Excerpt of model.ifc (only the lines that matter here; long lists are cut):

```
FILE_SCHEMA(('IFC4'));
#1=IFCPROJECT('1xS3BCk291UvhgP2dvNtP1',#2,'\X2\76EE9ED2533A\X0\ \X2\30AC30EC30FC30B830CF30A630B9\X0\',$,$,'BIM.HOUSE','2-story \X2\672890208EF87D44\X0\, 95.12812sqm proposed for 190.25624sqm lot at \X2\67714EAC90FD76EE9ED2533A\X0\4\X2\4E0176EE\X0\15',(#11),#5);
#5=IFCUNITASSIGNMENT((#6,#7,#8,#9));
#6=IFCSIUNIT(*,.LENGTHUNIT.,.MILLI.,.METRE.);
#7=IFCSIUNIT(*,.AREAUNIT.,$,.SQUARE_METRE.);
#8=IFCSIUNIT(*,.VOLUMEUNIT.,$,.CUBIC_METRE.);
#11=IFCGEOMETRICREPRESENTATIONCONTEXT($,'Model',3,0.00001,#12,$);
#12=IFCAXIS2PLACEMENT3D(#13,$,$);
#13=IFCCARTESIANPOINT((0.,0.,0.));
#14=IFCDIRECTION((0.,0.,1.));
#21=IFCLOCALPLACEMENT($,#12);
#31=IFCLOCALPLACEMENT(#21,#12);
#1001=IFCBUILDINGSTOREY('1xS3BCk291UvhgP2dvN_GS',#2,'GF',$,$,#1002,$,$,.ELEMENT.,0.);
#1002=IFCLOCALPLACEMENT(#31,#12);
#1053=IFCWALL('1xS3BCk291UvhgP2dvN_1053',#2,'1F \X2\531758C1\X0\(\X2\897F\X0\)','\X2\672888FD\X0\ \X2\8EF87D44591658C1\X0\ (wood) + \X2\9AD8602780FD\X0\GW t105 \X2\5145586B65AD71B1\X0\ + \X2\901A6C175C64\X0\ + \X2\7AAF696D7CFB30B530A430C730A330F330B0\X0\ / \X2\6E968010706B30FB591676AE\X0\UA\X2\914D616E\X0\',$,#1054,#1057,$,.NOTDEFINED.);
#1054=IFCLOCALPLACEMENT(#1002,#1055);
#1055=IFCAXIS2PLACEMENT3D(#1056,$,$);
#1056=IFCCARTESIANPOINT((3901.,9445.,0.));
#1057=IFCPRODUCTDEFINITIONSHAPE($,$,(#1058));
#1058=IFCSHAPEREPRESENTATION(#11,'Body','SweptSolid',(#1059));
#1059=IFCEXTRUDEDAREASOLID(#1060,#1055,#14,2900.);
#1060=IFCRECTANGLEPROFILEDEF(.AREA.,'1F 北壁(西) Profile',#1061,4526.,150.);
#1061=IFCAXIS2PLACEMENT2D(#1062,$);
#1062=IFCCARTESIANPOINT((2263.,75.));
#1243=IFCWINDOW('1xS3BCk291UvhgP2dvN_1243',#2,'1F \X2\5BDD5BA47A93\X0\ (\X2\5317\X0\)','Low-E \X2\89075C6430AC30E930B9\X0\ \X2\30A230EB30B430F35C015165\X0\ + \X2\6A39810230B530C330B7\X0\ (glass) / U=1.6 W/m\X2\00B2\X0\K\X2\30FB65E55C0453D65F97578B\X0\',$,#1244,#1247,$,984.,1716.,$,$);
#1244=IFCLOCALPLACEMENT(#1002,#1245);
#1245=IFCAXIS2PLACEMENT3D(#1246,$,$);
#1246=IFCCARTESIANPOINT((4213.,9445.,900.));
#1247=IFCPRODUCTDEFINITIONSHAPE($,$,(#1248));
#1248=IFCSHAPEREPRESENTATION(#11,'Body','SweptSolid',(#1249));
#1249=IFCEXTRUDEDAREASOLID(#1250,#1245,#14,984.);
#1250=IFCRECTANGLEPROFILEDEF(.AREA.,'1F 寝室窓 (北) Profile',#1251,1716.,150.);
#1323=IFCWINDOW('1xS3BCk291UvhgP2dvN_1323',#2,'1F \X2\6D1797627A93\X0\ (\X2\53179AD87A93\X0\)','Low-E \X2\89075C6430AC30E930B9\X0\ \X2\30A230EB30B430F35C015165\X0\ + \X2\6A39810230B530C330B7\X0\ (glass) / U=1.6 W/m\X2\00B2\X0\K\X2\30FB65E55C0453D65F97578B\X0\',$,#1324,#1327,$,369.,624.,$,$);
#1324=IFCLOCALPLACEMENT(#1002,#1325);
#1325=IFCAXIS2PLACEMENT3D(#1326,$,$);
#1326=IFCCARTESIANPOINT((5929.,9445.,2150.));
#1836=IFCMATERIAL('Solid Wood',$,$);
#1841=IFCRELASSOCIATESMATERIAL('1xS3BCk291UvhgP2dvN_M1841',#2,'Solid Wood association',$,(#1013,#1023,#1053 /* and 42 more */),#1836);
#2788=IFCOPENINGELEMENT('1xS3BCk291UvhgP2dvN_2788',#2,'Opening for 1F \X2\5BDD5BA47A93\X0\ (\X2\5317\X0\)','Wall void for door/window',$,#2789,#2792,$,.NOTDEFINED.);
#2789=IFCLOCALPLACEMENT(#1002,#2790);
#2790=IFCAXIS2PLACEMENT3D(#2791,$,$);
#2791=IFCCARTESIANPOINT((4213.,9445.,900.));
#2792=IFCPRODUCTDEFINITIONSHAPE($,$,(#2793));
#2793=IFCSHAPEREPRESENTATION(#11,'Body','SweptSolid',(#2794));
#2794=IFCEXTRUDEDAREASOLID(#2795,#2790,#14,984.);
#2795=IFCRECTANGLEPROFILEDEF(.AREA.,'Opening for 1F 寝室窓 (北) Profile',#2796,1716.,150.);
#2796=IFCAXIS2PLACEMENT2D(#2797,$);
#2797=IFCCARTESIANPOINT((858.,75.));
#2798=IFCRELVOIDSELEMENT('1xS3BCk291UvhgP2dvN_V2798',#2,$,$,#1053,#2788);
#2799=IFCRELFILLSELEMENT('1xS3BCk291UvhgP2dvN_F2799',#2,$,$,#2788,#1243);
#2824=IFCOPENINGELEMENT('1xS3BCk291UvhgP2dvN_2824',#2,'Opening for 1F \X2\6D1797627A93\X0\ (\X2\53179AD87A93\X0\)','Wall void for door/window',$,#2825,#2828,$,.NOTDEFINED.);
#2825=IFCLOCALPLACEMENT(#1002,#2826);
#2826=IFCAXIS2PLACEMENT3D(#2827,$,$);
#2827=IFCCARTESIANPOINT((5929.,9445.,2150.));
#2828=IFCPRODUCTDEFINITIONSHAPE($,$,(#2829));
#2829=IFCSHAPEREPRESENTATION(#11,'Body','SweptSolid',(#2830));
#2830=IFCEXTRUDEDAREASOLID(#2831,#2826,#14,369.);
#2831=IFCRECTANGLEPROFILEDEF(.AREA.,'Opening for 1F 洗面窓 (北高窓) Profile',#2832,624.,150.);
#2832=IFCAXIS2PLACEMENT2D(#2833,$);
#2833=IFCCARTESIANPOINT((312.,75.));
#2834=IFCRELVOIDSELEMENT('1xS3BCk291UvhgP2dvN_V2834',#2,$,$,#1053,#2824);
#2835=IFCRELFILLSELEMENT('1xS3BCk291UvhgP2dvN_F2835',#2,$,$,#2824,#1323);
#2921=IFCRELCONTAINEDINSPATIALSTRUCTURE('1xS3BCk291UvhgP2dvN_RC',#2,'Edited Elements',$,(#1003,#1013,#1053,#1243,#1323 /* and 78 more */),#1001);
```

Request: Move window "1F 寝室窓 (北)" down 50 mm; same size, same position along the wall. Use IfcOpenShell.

```python
import numpy as np
import ifcopenshell
import ifcopenshell.api.geometry
import ifcopenshell.util.placement
import ifcopenshell.util.unit

model = ifcopenshell.open("model.ifc")
unit_scale = ifcopenshell.util.unit.calculate_unit_scale(model)

window = model.by_guid("1xS3BCk291UvhgP2dvN_1243")
opening = window.FillsVoids[0].RelatingOpeningElement
dz = -0.05 / unit_scale

shift = np.array([0.0, 0.0, dz])
# The window is not placed relative to its opening, so move both.
for product in (opening, window):
    matrix = ifcopenshell.util.placement.get_local_placement(product.ObjectPlacement)
    matrix[:3, 3] += shift
    ifcopenshell.api.geometry.edit_object_placement(model, product=product, matrix=matrix, is_si=False)

print(f"moved by {dz * unit_scale:+.3f} m")

model.write("model_v2.ifc")
```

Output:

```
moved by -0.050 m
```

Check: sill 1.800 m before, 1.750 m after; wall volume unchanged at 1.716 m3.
